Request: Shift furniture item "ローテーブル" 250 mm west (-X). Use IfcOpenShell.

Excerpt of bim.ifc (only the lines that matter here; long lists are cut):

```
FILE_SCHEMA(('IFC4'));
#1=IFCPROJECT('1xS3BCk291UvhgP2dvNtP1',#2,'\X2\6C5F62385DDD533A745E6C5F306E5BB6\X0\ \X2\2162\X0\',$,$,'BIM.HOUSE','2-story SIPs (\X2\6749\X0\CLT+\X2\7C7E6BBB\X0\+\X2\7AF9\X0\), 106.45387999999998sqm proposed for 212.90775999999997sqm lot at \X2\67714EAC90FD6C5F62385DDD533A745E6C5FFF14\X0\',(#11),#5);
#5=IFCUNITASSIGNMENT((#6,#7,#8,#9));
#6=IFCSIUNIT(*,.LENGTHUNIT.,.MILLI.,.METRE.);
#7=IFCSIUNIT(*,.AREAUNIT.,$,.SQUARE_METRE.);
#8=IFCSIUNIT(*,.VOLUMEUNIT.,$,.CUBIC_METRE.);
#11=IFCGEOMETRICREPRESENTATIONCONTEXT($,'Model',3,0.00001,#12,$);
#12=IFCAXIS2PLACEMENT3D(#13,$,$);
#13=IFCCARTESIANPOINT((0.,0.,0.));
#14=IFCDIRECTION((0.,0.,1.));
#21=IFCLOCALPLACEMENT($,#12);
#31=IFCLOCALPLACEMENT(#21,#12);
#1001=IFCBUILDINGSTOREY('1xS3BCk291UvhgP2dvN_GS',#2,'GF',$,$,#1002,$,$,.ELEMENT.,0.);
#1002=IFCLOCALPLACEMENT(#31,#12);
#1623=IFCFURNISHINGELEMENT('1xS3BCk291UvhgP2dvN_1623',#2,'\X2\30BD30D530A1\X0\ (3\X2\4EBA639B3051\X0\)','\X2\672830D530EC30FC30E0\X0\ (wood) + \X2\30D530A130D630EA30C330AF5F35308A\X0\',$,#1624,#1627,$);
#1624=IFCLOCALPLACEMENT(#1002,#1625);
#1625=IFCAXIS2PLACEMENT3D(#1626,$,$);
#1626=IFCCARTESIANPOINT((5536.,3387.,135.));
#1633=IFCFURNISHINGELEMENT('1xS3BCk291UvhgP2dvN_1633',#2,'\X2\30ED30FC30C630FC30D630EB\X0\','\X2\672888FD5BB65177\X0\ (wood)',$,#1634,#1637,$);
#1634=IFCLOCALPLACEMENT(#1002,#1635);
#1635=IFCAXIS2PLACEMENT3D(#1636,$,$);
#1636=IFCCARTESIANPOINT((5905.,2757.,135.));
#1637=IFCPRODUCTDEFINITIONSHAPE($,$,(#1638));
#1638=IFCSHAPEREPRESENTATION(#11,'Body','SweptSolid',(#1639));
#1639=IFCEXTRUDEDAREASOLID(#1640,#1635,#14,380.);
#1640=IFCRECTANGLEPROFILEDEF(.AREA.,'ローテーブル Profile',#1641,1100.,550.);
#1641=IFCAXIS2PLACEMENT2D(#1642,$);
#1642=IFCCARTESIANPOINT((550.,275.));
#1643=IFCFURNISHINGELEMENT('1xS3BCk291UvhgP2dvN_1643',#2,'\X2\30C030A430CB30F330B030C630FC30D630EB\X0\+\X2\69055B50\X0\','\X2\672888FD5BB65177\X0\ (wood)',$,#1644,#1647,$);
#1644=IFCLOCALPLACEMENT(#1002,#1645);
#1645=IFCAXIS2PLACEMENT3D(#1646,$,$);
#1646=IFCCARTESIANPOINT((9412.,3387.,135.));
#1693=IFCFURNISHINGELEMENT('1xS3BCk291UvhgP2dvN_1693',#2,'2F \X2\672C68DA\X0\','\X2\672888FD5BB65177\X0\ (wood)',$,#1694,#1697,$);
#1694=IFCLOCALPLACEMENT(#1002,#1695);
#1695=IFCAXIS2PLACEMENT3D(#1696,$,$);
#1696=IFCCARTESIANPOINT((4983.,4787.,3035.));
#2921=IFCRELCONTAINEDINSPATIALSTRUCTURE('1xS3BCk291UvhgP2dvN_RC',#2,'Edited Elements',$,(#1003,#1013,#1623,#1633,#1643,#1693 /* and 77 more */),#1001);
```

```python
import ifcopenshell
import ifcopenshell.api.geometry
import ifcopenshell.util.placement
import ifcopenshell.util.unit

model = ifcopenshell.open("bim.ifc")
unit_scale = ifcopenshell.util.unit.calculate_unit_scale(model)

item = model.by_id(1633)
matrix = ifcopenshell.util.placement.get_local_placement(item.ObjectPlacement)
matrix[0, 3] -= 0.25 / unit_scale
ifcopenshell.api.geometry.edit_object_placement(model, product=item, matrix=matrix, is_si=False)

print(ifcopenshell.util.placement.get_local_placement(item.ObjectPlacement).round(3) + 0.0)

model.write("bim_edited.ifc")
```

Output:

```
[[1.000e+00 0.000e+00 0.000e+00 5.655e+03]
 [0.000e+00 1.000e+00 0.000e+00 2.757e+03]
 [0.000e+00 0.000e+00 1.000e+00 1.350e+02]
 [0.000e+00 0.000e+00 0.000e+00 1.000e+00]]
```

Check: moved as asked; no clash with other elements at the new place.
